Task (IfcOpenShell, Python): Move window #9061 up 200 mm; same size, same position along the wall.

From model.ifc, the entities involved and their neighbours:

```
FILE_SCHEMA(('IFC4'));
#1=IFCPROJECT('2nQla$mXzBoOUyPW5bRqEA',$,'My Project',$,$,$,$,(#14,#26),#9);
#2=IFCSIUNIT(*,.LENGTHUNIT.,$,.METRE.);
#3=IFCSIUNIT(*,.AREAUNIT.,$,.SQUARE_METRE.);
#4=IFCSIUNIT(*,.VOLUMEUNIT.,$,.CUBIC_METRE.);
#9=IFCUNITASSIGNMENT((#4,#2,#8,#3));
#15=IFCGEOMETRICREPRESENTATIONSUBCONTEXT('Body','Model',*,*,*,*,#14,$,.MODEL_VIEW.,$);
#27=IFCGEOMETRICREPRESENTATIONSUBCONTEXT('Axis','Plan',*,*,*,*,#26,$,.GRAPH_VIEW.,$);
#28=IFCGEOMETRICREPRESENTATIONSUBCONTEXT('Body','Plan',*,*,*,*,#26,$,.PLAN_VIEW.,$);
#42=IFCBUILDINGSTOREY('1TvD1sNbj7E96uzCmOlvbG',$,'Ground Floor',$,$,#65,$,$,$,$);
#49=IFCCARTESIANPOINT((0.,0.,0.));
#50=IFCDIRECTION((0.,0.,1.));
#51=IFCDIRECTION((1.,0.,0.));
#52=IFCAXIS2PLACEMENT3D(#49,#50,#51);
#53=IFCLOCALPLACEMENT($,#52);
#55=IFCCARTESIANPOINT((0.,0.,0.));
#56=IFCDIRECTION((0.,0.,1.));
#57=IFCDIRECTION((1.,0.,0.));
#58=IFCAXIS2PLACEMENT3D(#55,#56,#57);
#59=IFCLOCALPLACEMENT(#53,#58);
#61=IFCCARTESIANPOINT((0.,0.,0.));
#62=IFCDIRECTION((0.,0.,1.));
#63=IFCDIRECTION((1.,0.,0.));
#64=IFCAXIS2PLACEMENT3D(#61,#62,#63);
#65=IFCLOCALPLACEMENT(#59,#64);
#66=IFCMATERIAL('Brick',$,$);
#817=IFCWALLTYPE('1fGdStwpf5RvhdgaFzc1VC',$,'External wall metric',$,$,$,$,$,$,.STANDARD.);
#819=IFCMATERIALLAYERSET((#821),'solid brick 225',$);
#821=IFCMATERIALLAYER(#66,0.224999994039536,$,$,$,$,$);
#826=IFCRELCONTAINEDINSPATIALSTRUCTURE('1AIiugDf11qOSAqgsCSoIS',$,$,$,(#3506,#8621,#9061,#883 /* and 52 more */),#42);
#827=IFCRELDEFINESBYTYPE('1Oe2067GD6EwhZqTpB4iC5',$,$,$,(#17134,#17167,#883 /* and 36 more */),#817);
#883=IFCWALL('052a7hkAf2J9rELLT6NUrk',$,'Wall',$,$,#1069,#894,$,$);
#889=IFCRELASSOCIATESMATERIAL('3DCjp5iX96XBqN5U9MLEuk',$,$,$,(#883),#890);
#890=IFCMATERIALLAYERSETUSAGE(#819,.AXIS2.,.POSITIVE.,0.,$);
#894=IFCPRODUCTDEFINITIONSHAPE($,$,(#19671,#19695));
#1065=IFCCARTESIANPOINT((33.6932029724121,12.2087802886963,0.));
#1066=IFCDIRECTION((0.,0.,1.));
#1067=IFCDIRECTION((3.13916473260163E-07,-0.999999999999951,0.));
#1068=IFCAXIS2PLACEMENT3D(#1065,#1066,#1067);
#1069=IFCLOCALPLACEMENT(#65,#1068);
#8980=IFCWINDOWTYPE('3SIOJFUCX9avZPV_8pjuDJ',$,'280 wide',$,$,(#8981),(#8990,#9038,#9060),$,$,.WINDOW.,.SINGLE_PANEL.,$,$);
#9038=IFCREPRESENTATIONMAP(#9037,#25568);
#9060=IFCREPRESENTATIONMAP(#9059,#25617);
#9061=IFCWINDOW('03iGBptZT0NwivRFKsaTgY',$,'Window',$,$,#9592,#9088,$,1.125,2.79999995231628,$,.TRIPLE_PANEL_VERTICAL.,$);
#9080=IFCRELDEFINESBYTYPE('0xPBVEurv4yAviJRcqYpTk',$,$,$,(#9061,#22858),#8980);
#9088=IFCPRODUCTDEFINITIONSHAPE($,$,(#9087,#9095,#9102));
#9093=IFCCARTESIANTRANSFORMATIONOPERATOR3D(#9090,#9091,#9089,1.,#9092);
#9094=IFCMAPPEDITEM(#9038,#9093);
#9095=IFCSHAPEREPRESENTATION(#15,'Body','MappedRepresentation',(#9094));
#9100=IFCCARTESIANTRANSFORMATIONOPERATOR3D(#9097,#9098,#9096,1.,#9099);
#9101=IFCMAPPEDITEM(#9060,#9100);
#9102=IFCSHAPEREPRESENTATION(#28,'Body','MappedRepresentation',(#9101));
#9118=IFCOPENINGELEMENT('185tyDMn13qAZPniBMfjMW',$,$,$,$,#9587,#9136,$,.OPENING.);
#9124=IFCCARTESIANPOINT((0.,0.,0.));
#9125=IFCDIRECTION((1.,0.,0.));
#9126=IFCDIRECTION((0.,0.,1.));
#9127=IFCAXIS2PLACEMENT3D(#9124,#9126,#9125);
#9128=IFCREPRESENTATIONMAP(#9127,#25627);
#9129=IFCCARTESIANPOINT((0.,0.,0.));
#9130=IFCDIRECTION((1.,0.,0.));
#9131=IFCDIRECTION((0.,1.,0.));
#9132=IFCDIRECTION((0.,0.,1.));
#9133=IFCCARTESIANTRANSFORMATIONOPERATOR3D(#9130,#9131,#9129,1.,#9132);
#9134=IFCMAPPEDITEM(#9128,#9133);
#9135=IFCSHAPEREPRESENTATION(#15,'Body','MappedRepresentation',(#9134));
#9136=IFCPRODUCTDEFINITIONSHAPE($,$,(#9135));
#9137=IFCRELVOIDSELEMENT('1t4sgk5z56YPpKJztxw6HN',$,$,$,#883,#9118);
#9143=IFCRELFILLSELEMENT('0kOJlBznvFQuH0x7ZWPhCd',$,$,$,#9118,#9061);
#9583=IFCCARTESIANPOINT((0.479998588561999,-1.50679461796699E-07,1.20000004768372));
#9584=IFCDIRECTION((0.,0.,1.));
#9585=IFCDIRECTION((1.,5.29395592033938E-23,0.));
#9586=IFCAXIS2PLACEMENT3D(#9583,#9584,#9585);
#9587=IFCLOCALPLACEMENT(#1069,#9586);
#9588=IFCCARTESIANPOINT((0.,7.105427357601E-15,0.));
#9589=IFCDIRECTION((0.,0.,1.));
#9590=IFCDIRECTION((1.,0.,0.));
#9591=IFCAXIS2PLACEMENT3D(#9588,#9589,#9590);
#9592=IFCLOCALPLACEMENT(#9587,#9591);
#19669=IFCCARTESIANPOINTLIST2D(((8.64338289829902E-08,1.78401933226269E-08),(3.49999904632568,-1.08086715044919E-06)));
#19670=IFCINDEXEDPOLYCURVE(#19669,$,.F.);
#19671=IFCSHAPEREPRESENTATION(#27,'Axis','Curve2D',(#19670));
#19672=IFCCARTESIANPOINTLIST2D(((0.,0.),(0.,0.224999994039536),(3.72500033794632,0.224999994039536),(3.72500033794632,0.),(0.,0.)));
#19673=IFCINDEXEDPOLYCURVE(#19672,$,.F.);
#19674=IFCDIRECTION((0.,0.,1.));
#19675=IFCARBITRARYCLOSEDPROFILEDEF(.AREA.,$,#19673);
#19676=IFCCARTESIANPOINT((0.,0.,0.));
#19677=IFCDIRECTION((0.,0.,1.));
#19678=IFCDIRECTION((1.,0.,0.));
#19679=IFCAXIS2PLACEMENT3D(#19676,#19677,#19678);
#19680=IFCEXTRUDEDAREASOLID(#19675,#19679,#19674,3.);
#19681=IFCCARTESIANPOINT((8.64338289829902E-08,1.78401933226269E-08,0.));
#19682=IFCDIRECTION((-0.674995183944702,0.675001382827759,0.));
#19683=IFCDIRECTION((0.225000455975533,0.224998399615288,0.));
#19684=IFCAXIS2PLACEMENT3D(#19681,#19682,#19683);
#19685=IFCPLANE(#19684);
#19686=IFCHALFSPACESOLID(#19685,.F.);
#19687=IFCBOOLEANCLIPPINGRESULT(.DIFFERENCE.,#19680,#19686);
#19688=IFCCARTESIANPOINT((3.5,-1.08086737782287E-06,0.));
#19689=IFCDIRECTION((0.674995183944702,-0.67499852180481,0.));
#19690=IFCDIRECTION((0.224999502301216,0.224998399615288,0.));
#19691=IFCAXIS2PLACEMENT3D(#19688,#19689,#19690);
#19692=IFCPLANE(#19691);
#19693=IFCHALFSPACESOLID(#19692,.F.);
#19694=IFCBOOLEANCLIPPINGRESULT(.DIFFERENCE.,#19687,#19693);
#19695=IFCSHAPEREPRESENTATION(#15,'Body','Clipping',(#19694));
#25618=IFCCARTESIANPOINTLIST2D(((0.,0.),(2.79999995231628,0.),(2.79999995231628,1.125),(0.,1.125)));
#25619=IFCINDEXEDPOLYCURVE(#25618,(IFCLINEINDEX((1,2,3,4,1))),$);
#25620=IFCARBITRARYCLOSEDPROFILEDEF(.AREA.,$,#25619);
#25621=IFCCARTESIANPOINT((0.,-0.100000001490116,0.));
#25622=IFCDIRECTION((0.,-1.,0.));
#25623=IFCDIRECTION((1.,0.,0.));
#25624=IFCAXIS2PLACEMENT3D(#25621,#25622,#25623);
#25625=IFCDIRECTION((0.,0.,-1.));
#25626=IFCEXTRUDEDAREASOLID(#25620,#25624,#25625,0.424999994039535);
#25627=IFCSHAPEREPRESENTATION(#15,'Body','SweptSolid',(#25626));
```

```python
import numpy as np
import ifcopenshell
import ifcopenshell.api.geometry
import ifcopenshell.util.placement
import ifcopenshell.util.unit

model = ifcopenshell.open("model.ifc")
unit_scale = ifcopenshell.util.unit.calculate_unit_scale(model)

window = model.by_guid("03iGBptZT0NwivRFKsaTgY")
opening = window.FillsVoids[0].RelatingOpeningElement
dz = 0.2 / unit_scale

shift = np.array([0.0, 0.0, dz])
# The window is placed relative to its opening, so it follows when the opening moves.
matrix = ifcopenshell.util.placement.get_local_placement(opening.ObjectPlacement)
matrix[:3, 3] += shift
ifcopenshell.api.geometry.edit_object_placement(
    model, product=opening, matrix=matrix, is_si=False, should_transform_children=True
)

print(f"moved by {dz * unit_scale:+.3f} m")

model.write("model_updated.ifc")
```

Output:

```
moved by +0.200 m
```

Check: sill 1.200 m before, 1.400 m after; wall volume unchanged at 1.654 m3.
